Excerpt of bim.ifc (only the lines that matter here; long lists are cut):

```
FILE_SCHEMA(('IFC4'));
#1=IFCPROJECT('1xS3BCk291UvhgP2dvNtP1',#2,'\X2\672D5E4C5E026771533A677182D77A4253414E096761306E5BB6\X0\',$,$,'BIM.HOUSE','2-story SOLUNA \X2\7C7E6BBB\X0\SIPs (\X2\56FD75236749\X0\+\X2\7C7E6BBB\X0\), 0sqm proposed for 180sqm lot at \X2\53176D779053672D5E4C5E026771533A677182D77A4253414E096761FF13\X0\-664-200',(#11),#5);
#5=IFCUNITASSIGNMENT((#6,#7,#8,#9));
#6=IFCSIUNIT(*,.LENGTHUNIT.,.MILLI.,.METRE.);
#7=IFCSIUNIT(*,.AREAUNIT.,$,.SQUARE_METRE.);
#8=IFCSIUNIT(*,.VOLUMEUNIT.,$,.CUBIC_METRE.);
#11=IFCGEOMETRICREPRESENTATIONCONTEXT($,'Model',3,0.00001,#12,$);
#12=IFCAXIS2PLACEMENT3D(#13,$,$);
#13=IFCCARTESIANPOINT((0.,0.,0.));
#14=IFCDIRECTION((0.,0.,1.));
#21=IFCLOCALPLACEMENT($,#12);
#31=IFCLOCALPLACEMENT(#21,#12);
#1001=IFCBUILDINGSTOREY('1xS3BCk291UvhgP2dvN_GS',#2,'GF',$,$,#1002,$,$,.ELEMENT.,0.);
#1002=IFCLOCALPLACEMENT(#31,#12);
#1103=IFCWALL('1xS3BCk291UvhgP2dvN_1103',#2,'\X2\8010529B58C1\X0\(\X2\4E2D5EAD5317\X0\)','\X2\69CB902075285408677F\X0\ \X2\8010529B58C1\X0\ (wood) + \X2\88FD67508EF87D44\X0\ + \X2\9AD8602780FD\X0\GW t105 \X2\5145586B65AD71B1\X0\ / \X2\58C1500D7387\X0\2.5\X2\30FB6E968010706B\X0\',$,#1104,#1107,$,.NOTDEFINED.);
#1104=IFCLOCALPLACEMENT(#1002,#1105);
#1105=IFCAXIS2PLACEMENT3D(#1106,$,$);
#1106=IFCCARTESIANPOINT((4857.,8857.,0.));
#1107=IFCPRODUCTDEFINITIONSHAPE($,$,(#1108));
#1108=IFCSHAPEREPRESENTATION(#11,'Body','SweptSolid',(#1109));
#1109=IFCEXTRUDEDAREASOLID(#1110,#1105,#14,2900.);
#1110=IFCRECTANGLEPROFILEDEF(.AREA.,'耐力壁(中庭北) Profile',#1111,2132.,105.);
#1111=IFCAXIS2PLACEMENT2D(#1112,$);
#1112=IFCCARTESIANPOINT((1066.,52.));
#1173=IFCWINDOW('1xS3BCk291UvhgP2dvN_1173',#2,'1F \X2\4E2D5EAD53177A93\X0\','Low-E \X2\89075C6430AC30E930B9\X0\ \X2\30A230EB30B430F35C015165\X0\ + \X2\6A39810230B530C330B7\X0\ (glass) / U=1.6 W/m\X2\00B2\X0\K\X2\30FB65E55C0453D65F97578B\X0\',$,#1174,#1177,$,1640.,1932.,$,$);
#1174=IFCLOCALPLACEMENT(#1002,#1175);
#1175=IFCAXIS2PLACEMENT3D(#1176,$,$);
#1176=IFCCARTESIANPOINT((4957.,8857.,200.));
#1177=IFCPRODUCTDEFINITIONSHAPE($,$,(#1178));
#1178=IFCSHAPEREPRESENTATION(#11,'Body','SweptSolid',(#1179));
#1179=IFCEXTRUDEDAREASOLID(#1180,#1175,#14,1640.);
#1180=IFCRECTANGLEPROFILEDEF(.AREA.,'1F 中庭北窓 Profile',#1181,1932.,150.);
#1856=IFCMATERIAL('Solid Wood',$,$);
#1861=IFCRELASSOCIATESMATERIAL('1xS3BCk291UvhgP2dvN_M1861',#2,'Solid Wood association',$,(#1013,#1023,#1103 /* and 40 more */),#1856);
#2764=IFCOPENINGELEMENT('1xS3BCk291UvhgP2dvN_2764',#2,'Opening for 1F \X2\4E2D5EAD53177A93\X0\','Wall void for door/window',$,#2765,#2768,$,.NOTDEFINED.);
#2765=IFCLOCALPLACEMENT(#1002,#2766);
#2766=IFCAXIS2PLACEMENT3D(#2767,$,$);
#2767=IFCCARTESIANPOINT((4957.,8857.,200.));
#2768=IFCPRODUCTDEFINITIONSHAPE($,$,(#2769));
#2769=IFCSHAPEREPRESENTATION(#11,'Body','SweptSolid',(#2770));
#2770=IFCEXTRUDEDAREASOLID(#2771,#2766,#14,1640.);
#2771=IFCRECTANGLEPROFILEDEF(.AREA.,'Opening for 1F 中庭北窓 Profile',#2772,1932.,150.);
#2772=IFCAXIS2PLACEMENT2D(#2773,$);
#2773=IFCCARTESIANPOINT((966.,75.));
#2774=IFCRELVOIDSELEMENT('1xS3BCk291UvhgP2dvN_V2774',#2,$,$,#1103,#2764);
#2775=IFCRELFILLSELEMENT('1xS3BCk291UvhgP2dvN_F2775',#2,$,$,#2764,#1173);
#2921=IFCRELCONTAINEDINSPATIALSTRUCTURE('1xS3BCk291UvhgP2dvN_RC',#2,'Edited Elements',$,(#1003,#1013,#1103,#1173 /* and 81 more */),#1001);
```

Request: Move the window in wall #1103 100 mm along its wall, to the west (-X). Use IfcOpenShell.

```python
import ifcopenshell
import ifcopenshell.api.geometry
import ifcopenshell.util.placement
import ifcopenshell.util.unit

model = ifcopenshell.open("bim.ifc")
unit_scale = ifcopenshell.util.unit.calculate_unit_scale(model)

window = model.by_id(1173)
opening = window.FillsVoids[0].RelatingOpeningElement
wall = opening.VoidsElements[0].RelatingBuildingElement

wall_matrix = ifcopenshell.util.placement.get_local_placement(wall.ObjectPlacement)
shift = wall_matrix[:3, 0] * -0.1 / unit_scale
before = ifcopenshell.util.placement.get_local_placement(window.ObjectPlacement)[:3, 3].copy()

# The window is not placed relative to its opening, so move both.
for product in (opening, window):
    matrix = ifcopenshell.util.placement.get_local_placement(product.ObjectPlacement)
    matrix[:3, 3] += shift
    ifcopenshell.api.geometry.edit_object_placement(model, product=product, matrix=matrix, is_si=False)

after = ifcopenshell.util.placement.get_local_placement(window.ObjectPlacement)[:3, 3]
print("window moved by", (after - before).round(3) + 0.0)

model.write("bim_v2.ifc")
```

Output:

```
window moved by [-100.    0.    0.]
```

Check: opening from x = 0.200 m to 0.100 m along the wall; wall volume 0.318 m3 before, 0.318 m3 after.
